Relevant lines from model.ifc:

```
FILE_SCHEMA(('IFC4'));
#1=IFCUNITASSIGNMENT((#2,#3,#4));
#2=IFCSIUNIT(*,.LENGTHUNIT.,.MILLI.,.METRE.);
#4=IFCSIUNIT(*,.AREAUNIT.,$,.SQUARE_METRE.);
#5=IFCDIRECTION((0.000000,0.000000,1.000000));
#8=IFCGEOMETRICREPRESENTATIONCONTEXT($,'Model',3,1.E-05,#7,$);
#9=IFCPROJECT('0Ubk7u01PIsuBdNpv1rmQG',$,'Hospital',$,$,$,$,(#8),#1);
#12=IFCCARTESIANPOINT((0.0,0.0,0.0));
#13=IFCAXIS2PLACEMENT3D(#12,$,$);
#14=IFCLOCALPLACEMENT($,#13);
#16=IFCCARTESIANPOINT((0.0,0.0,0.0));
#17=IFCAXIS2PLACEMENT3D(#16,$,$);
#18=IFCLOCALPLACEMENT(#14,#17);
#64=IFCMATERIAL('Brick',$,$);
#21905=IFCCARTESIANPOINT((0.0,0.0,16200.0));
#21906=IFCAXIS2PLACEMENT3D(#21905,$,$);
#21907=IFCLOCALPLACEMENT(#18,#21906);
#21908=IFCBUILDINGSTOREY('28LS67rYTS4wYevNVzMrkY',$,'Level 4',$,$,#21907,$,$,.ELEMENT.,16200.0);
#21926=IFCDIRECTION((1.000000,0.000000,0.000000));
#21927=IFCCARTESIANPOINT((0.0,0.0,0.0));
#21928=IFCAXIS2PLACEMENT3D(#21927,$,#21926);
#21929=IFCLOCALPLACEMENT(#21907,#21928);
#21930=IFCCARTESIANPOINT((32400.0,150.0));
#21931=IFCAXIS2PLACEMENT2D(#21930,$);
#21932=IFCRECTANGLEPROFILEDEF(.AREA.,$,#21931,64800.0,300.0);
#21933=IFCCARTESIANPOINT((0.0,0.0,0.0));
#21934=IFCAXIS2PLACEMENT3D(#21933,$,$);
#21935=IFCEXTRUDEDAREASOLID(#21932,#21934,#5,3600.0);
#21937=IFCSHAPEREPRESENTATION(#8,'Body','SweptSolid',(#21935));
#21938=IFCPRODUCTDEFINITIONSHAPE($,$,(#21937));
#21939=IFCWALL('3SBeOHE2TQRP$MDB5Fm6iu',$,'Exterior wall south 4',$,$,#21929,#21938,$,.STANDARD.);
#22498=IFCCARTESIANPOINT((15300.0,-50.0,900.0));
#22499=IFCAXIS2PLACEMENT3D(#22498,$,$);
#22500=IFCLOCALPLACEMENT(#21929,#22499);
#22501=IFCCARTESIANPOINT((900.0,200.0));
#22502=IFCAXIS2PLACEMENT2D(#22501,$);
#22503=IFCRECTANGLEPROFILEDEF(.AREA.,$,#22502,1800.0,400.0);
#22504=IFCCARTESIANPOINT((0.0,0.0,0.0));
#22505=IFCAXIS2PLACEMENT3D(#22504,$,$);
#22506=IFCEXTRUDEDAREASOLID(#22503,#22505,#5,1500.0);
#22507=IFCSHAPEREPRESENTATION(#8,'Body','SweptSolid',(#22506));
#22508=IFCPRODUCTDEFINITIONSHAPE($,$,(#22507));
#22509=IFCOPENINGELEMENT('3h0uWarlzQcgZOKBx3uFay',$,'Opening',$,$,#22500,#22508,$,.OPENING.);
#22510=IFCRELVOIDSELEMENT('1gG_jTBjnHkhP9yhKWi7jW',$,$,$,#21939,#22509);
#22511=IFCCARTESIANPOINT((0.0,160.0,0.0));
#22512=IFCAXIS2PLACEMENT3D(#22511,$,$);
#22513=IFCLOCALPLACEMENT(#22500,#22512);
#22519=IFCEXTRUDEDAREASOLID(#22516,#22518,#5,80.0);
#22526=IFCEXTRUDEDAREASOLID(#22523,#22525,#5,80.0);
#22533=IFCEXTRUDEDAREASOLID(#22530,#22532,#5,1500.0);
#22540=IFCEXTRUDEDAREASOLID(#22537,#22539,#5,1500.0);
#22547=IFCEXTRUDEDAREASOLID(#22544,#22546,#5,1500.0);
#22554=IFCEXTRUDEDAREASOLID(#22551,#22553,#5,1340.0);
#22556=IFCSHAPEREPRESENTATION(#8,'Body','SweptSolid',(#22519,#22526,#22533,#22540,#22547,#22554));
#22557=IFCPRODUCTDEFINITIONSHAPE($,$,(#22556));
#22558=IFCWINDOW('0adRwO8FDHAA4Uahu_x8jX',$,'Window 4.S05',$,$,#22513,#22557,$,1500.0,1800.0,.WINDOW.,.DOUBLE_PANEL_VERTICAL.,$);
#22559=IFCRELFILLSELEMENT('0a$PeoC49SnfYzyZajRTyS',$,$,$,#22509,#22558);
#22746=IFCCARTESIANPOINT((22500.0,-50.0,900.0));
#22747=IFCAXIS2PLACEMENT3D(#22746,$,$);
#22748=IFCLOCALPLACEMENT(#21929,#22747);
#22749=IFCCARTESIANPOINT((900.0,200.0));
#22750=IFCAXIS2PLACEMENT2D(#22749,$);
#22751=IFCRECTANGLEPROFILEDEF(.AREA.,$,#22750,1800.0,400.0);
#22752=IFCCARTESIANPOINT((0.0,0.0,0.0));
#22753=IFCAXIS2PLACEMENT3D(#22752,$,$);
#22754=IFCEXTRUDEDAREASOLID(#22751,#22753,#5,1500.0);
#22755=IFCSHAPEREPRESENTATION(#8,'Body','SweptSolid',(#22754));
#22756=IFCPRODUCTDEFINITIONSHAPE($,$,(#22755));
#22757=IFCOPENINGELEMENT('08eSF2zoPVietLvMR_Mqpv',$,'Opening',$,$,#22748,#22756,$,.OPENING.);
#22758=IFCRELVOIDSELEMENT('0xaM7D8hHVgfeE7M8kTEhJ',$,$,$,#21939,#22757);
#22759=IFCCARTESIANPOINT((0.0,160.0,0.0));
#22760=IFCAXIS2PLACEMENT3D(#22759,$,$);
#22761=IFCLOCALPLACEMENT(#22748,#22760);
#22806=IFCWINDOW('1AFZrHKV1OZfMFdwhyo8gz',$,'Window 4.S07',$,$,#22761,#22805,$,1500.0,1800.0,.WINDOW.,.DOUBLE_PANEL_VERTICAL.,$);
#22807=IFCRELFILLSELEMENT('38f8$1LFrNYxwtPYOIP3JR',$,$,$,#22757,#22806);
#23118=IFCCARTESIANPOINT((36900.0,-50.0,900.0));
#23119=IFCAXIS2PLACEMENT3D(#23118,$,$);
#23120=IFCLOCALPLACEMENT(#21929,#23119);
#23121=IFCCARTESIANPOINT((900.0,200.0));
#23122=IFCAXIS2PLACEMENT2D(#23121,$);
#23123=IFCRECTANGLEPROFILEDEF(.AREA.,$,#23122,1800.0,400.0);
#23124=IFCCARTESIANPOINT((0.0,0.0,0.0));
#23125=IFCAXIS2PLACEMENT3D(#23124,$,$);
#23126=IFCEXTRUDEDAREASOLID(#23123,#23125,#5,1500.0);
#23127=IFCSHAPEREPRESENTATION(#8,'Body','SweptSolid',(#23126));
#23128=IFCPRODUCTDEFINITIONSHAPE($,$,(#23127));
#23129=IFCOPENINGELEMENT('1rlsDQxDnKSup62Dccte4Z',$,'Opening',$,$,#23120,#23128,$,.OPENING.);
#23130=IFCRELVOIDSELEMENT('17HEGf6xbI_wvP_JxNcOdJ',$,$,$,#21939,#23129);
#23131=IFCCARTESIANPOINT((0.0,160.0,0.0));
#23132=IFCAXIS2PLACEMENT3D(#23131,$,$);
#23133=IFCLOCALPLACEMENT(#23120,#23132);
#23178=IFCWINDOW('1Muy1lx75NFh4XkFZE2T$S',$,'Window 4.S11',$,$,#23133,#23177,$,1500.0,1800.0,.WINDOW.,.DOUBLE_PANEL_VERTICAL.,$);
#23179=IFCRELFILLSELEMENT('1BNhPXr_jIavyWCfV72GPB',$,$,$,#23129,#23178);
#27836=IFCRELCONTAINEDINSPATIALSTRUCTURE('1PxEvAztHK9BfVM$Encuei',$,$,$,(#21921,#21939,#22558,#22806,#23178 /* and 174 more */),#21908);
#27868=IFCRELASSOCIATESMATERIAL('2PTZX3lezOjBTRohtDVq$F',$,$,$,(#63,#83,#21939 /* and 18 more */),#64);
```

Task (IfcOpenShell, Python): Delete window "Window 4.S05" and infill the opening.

```python
import ifcopenshell
import ifcopenshell.api.feature
import ifcopenshell.api.root
import ifcopenshell.geom
import ifcopenshell.util.shape

model = ifcopenshell.open("model.ifc")
settings = ifcopenshell.geom.settings()


def volume(element):
    """Net volume in cubic metres, openings subtracted."""
    shape = ifcopenshell.geom.create_shape(settings, element)
    return ifcopenshell.util.shape.get_volume(shape.geometry)


window = model.by_guid("0adRwO8FDHAA4Uahu_x8jX")
opening = window.FillsVoids[0].RelatingOpeningElement
wall = opening.VoidsElements[0].RelatingBuildingElement
before = volume(wall)

ifcopenshell.api.root.remove_product(model, product=window)
ifcopenshell.api.feature.remove_feature(model, feature=opening)

after = volume(wall)

print(f"wall volume {before:.3f} -> {after:.3f} m3")

model.write("model-out.ifc")
```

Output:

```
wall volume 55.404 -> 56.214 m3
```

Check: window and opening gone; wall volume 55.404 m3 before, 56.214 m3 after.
